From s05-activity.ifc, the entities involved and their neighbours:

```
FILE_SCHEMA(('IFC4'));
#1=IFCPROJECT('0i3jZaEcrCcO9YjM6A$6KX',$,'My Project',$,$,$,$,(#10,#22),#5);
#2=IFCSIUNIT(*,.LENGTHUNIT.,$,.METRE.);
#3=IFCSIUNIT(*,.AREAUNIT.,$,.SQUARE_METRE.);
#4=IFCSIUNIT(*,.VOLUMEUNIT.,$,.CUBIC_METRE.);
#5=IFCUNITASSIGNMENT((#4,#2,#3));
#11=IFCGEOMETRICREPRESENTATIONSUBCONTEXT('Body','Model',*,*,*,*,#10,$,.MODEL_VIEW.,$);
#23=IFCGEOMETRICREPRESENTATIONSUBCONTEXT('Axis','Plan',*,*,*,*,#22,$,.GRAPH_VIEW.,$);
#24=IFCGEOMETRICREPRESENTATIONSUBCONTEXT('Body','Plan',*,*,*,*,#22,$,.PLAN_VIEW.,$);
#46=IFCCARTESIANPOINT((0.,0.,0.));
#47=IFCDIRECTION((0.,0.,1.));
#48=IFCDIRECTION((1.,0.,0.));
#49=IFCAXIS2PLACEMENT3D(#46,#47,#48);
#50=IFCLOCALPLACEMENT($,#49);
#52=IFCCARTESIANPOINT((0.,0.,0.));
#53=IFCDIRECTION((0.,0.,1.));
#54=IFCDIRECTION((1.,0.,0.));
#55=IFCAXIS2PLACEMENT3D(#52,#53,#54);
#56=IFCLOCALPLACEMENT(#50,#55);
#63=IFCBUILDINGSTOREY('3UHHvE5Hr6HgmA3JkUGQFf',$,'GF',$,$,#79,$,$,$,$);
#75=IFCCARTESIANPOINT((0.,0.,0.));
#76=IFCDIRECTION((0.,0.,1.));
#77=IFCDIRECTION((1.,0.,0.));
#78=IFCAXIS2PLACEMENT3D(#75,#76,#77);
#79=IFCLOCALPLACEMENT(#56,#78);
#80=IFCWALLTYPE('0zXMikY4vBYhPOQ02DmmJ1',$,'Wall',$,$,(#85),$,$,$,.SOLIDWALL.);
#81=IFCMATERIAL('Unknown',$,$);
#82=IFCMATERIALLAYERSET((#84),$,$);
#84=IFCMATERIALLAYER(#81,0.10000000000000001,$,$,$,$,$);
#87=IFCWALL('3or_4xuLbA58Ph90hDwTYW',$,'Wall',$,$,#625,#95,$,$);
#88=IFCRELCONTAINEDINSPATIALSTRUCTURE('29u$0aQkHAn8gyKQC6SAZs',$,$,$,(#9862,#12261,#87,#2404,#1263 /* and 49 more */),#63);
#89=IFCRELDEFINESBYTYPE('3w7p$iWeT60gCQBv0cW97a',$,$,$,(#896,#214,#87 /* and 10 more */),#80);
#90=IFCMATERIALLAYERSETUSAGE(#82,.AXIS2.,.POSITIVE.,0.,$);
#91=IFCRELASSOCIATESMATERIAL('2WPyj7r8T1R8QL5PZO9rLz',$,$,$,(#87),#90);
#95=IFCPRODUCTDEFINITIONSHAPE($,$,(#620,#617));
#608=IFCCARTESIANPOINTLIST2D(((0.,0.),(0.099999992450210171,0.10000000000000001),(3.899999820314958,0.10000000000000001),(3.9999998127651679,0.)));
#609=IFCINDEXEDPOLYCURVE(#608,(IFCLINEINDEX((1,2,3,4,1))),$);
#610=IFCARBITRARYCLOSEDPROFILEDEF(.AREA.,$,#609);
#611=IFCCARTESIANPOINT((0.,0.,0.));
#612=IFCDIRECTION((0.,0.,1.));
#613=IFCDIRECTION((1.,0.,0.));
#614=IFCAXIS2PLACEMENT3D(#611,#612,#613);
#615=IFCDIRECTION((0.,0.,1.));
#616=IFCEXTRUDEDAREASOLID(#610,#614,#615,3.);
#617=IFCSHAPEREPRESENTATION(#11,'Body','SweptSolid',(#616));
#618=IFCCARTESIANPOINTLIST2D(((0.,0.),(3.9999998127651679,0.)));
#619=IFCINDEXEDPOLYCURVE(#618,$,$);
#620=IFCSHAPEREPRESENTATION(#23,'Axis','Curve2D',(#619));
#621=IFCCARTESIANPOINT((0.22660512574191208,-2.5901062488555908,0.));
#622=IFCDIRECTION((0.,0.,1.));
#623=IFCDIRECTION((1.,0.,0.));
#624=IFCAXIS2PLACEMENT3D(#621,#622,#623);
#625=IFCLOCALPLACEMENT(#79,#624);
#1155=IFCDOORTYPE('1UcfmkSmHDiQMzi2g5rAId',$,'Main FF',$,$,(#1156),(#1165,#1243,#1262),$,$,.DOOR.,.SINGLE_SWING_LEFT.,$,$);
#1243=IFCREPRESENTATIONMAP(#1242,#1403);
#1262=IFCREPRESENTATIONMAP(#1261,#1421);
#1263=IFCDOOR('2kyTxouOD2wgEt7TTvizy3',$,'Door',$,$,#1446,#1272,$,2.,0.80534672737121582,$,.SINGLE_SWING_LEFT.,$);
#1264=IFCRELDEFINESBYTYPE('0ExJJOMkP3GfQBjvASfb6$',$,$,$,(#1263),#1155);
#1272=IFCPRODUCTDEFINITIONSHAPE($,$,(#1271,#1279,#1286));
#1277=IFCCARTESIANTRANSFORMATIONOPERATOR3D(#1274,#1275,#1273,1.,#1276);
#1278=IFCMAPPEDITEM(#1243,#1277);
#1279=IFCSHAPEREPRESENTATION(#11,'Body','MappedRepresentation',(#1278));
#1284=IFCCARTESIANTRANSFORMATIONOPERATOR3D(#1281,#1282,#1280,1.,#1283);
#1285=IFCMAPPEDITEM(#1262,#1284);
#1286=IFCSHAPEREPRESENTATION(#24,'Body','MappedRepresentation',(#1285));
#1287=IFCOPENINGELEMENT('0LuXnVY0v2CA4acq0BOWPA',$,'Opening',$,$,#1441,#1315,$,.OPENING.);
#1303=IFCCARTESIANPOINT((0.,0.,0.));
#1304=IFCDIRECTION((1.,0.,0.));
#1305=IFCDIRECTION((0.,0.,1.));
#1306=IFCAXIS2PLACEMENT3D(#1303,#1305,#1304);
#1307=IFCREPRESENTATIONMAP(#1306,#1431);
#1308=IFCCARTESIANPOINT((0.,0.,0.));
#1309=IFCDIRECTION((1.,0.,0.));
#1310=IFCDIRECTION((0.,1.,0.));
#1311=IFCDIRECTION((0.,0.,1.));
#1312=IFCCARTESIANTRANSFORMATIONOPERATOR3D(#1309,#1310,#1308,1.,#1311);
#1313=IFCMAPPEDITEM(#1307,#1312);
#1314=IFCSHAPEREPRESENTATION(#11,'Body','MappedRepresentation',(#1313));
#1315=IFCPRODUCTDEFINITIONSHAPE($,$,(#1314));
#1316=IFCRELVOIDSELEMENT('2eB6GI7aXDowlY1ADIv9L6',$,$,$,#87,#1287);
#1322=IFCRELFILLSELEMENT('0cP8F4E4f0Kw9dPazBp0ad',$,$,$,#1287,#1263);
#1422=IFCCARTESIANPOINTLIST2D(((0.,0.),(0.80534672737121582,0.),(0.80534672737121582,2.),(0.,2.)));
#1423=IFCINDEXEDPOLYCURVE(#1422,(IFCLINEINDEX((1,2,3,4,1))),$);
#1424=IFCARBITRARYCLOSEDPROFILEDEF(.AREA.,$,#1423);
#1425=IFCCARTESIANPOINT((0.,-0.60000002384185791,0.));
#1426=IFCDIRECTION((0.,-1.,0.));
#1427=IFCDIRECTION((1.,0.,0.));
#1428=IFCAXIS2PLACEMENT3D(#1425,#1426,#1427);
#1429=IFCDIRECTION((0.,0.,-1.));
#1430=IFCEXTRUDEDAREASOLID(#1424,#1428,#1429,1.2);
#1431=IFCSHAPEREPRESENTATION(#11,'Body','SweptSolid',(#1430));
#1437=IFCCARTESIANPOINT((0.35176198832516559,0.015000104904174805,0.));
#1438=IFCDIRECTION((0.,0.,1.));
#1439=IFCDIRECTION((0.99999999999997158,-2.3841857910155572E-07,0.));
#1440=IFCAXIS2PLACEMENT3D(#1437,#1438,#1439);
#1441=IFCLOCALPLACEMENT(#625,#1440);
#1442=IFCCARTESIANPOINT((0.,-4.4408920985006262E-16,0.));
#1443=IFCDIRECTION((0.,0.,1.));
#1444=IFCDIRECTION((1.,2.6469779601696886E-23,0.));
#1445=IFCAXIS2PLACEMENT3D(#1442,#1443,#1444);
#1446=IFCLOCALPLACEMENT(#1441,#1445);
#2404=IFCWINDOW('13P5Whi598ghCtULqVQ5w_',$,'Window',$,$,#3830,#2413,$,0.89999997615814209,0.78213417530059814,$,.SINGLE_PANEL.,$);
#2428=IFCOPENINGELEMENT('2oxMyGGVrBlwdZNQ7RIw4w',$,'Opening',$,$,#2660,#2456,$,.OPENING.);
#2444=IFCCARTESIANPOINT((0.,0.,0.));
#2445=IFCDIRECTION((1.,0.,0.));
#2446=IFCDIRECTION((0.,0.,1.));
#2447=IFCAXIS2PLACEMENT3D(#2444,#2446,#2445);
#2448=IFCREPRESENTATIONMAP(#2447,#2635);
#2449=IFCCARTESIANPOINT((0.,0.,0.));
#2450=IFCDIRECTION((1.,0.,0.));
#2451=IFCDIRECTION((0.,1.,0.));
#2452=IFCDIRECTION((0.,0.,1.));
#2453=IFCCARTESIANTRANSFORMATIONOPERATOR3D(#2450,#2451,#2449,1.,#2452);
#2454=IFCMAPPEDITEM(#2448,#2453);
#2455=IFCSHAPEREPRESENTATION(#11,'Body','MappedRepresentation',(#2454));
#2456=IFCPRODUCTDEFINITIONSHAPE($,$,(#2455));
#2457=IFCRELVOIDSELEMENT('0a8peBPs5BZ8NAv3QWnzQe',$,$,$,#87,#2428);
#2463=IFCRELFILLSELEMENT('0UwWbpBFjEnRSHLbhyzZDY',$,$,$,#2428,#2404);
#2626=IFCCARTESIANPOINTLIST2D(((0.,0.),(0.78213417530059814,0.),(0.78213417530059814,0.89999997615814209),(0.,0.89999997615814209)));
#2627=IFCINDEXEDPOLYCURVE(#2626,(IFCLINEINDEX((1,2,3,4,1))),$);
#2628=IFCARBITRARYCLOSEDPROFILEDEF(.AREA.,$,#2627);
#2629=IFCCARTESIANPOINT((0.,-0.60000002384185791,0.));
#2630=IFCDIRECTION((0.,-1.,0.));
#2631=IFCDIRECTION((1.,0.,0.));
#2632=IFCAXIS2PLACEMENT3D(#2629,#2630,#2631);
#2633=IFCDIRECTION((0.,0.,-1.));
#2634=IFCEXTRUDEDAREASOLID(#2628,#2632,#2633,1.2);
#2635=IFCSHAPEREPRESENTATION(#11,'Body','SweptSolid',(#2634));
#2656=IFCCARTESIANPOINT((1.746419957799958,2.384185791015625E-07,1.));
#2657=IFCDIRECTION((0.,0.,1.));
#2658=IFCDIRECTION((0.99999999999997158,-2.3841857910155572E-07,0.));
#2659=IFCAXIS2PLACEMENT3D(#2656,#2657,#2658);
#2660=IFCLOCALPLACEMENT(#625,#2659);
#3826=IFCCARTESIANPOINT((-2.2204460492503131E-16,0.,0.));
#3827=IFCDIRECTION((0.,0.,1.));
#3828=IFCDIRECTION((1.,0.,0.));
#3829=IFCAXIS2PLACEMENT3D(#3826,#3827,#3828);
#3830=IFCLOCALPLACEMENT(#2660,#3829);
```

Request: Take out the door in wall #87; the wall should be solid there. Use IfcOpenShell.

```python
import ifcopenshell
import ifcopenshell.api.feature
import ifcopenshell.api.root
import ifcopenshell.geom
import ifcopenshell.util.shape

model = ifcopenshell.open("s05-activity.ifc")
settings = ifcopenshell.geom.settings()


def volume(element):
    """Net volume in cubic metres, openings subtracted."""
    shape = ifcopenshell.geom.create_shape(settings, element)
    return ifcopenshell.util.shape.get_volume(shape.geometry)


door = model.by_guid("2kyTxouOD2wgEt7TTvizy3")
opening = door.FillsVoids[0].RelatingOpeningElement
wall = opening.VoidsElements[0].RelatingBuildingElement
before = volume(wall)

ifcopenshell.api.root.remove_product(model, product=door)
ifcopenshell.api.feature.remove_feature(model, feature=opening)

after = volume(wall)

print(f"wall volume {before:.3f} -> {after:.3f} m3")

model.write("s05-activity_v2.ifc")
```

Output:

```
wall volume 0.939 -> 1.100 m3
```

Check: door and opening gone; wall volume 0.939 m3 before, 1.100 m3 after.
